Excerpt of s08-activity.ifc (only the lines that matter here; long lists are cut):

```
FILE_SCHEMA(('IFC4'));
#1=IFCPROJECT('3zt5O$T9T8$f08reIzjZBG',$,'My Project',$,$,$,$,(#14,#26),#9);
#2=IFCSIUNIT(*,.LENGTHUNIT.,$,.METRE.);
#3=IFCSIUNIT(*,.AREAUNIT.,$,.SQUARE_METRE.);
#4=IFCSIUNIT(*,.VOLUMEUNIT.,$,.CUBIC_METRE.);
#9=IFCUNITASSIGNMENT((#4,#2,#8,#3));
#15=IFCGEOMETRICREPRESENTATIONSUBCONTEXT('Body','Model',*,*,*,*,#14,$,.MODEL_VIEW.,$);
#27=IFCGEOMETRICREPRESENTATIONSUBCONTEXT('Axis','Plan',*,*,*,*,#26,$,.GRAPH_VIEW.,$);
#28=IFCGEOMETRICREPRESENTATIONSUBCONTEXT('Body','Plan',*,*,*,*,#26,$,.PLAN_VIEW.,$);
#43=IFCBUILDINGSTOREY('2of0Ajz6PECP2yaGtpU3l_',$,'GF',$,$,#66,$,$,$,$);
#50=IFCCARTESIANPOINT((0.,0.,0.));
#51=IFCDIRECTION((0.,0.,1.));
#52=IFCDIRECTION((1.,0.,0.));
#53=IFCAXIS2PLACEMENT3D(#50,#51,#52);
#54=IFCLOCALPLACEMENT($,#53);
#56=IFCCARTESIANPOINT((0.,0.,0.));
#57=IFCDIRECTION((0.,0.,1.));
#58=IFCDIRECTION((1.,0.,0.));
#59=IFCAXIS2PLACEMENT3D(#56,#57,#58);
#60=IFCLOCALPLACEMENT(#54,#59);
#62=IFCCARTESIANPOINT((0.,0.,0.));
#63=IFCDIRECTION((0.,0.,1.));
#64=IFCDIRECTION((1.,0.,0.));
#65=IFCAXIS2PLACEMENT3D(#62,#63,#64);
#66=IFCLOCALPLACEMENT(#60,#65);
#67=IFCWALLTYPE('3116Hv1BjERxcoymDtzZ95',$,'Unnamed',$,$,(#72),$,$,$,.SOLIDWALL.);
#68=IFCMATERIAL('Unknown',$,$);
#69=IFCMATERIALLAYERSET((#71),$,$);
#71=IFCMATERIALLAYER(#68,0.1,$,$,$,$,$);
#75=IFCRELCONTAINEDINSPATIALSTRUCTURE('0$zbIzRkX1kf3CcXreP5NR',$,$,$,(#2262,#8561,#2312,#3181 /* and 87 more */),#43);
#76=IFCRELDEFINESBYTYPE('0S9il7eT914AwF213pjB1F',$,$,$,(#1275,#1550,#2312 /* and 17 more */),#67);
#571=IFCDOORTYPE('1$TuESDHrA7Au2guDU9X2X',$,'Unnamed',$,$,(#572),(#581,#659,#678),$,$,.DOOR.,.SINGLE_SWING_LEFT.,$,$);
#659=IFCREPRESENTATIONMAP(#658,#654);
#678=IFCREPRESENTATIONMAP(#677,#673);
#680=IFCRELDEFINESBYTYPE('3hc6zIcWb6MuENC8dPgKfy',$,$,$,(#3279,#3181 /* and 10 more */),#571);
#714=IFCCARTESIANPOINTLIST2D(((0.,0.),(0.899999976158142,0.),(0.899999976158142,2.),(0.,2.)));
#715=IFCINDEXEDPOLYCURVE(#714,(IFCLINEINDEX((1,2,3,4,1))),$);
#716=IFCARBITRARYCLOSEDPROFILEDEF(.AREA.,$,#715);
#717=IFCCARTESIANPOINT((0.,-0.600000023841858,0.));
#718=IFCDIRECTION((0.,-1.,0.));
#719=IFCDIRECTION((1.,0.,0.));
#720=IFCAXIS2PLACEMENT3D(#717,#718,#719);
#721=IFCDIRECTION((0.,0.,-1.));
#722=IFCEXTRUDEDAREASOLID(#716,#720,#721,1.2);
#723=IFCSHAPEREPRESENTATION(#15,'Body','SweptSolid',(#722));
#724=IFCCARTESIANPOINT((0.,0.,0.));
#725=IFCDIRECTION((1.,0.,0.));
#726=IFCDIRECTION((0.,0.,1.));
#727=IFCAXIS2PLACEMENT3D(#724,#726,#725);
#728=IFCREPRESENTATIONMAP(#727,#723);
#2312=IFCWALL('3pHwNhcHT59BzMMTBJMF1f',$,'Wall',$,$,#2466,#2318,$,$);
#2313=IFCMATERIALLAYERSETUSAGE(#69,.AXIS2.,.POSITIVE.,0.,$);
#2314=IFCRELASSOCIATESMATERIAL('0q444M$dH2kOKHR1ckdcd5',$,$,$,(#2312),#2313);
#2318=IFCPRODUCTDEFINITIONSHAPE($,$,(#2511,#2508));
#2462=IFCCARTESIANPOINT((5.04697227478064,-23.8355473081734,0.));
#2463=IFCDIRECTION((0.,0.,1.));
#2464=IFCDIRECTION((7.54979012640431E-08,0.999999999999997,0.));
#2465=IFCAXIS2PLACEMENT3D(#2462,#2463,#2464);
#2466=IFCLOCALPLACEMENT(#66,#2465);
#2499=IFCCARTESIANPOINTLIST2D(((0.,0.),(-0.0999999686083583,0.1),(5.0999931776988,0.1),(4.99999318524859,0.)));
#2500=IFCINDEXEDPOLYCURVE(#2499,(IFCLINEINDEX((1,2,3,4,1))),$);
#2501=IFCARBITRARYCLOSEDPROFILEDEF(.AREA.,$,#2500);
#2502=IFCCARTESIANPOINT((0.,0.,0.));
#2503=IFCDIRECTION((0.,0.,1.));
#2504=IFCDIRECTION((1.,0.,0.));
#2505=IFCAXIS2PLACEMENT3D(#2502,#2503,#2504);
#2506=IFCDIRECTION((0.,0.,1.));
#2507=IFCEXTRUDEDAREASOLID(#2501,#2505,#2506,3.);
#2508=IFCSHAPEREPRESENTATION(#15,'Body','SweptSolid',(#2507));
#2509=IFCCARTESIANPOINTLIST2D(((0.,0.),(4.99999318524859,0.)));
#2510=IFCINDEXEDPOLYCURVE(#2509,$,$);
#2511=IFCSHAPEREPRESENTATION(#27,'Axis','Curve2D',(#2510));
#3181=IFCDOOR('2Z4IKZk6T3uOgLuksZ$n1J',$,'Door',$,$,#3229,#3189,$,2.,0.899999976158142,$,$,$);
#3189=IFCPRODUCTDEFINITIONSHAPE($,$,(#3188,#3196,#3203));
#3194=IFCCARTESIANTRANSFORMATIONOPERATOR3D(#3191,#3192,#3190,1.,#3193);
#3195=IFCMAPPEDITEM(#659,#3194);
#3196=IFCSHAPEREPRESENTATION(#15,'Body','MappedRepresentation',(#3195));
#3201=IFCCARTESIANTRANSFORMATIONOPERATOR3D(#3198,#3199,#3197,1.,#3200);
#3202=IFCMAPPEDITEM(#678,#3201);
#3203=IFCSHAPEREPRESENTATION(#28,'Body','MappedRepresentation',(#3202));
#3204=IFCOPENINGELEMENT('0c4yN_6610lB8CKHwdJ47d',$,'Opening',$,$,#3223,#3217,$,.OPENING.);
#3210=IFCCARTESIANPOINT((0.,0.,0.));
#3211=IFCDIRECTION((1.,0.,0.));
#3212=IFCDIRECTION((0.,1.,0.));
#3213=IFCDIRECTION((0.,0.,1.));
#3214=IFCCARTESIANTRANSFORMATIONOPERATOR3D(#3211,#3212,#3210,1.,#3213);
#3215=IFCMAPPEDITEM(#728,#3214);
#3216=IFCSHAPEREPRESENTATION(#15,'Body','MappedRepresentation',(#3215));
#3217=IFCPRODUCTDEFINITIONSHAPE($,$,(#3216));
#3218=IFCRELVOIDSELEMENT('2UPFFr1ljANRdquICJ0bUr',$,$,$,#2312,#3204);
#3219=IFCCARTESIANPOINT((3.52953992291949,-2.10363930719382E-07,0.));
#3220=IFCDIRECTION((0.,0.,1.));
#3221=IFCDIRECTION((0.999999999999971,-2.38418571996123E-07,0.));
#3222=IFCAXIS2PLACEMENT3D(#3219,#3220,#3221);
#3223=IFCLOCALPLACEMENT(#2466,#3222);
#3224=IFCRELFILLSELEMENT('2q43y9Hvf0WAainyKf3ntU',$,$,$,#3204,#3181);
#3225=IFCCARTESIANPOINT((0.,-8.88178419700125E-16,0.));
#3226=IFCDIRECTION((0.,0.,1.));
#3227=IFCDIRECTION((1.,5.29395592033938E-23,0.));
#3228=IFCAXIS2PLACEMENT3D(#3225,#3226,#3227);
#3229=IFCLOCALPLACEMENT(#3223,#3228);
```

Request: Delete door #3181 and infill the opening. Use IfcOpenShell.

```python
import ifcopenshell
import ifcopenshell.api.feature
import ifcopenshell.api.root
import ifcopenshell.geom
import ifcopenshell.util.shape

model = ifcopenshell.open("s08-activity.ifc")
settings = ifcopenshell.geom.settings()


def volume(element):
    """Net volume in cubic metres, openings subtracted."""
    shape = ifcopenshell.geom.create_shape(settings, element)
    return ifcopenshell.util.shape.get_volume(shape.geometry)


door = model.by_guid("2Z4IKZk6T3uOgLuksZ$n1J")
opening = door.FillsVoids[0].RelatingOpeningElement
wall = opening.VoidsElements[0].RelatingBuildingElement
before = volume(wall)

ifcopenshell.api.root.remove_product(model, product=door)
ifcopenshell.api.feature.remove_feature(model, feature=opening)

after = volume(wall)

print(f"wall volume {before:.3f} -> {after:.3f} m3")

model.write("s08-activity_rev.ifc")
```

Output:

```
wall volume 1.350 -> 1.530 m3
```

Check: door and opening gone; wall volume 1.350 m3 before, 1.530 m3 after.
